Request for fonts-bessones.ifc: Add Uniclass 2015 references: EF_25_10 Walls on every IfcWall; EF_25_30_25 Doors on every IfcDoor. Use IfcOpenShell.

First a look at what the model holds.

```python
import ifcopenshell

model = ifcopenshell.open("fonts-bessones.ifc")
print(model.schema)
print("classifications:", [c.Name for c in model.by_type("IfcClassification")])
for ifc_class in ("IfcDoor", "IfcRoof", "IfcStair", "IfcWall", "IfcWindow"):
    print(ifc_class, len(model.by_type(ifc_class)))
```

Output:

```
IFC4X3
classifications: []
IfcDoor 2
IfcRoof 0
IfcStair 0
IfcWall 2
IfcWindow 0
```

```python
import ifcopenshell
import ifcopenshell.api.classification

model = ifcopenshell.open("fonts-bessones.ifc")

system = ifcopenshell.api.classification.add_classification(model, classification="Uniclass 2015")

codes = {
    "IfcWall": ("EF_25_10", "Walls"),
    "IfcDoor": ("EF_25_30_25", "Doors"),
}
for ifc_class, (code, name) in codes.items():
    products = model.by_type(ifc_class)
    ifcopenshell.api.classification.add_reference(
        model, products=products, classification=system, identification=code, name=name
    )
    print(code, len(products))

model.write("fonts-bessones_updated.ifc")
```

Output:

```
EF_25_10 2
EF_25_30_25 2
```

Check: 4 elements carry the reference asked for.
